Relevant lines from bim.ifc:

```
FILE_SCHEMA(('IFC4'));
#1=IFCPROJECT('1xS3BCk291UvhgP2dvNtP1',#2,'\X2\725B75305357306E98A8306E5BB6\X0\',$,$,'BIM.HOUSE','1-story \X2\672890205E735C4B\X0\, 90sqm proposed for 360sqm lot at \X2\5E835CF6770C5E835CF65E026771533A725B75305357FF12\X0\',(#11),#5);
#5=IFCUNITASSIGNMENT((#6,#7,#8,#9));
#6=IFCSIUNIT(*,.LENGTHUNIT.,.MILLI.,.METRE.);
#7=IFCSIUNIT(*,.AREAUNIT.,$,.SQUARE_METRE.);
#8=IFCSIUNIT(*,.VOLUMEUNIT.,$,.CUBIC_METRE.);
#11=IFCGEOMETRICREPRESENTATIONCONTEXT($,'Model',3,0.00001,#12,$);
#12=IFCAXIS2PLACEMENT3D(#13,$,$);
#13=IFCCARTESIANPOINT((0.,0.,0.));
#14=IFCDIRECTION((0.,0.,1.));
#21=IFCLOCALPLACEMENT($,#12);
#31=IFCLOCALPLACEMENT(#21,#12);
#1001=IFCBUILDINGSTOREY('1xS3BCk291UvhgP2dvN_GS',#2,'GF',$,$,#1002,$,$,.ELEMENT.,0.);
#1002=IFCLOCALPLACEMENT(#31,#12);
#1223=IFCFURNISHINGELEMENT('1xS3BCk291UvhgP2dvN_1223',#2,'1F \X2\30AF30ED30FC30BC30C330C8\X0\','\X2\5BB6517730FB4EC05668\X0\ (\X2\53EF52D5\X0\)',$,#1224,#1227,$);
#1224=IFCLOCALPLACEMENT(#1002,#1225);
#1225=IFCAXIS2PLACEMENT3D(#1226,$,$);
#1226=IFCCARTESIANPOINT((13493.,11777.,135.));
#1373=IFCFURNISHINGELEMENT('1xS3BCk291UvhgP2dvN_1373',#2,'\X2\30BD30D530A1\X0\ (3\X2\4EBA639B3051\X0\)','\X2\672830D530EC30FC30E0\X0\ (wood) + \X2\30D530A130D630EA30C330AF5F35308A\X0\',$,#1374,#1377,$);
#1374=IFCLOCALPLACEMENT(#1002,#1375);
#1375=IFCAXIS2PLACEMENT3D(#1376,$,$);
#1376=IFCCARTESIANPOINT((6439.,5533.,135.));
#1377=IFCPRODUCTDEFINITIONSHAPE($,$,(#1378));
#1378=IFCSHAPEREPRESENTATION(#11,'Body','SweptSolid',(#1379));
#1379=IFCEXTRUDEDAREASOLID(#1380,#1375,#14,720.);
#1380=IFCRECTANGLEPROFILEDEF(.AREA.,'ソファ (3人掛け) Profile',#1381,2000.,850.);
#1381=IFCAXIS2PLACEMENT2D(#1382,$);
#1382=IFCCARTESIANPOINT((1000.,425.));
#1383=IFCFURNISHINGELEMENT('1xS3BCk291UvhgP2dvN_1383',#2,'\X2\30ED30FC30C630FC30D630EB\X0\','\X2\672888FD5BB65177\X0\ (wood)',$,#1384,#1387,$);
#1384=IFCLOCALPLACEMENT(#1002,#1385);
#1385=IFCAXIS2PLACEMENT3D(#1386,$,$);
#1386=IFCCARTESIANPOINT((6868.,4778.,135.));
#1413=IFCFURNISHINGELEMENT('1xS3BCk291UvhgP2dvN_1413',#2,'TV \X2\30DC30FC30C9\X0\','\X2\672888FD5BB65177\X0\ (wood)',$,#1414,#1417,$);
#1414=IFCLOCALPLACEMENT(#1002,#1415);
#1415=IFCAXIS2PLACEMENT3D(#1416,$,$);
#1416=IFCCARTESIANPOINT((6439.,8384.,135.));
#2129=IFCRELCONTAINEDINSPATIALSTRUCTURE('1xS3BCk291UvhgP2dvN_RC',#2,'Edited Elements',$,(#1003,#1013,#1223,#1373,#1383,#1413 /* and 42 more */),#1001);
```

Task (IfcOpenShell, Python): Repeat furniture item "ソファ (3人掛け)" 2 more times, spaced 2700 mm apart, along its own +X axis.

```python
import ifcopenshell
import ifcopenshell.api.geometry
import ifcopenshell.api.root
import ifcopenshell.util.element
import ifcopenshell.util.placement

model = ifcopenshell.open("bim.ifc")


def reuse_history(source, copy):
    """copy_class also copies each property set's owner history, people and application; keep the originals."""
    for rel in copy.IsDefinedBy:
        if rel.is_a("IfcRelDefinesByProperties") and (history := rel.RelatingPropertyDefinition.OwnerHistory):
            rel.RelatingPropertyDefinition.OwnerHistory = source.OwnerHistory
            ifcopenshell.util.element.remove_deep2(model, history)


source = model.by_guid("1xS3BCk291UvhgP2dvN_1373")
base = ifcopenshell.util.placement.get_local_placement(source.ObjectPlacement)
step = base[:3, 0] * 2700.0

for i in range(1, 3):
    copy = ifcopenshell.api.root.copy_class(model, product=source)
    copy.Representation = ifcopenshell.util.element.copy_deep(
        model, source.Representation, exclude=["IfcGeometricRepresentationContext", "IfcRepresentationMap"]
    )
    reuse_history(source, copy)
    matrix = base.copy()
    matrix[:3, 3] += i * step
    print("added at", matrix[:3, 3].round(3) + 0.0)
    ifcopenshell.api.geometry.edit_object_placement(model, product=copy, matrix=matrix, is_si=False)

model.write("bim_rev.ifc")
```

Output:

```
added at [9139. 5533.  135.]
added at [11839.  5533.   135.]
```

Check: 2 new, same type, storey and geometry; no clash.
